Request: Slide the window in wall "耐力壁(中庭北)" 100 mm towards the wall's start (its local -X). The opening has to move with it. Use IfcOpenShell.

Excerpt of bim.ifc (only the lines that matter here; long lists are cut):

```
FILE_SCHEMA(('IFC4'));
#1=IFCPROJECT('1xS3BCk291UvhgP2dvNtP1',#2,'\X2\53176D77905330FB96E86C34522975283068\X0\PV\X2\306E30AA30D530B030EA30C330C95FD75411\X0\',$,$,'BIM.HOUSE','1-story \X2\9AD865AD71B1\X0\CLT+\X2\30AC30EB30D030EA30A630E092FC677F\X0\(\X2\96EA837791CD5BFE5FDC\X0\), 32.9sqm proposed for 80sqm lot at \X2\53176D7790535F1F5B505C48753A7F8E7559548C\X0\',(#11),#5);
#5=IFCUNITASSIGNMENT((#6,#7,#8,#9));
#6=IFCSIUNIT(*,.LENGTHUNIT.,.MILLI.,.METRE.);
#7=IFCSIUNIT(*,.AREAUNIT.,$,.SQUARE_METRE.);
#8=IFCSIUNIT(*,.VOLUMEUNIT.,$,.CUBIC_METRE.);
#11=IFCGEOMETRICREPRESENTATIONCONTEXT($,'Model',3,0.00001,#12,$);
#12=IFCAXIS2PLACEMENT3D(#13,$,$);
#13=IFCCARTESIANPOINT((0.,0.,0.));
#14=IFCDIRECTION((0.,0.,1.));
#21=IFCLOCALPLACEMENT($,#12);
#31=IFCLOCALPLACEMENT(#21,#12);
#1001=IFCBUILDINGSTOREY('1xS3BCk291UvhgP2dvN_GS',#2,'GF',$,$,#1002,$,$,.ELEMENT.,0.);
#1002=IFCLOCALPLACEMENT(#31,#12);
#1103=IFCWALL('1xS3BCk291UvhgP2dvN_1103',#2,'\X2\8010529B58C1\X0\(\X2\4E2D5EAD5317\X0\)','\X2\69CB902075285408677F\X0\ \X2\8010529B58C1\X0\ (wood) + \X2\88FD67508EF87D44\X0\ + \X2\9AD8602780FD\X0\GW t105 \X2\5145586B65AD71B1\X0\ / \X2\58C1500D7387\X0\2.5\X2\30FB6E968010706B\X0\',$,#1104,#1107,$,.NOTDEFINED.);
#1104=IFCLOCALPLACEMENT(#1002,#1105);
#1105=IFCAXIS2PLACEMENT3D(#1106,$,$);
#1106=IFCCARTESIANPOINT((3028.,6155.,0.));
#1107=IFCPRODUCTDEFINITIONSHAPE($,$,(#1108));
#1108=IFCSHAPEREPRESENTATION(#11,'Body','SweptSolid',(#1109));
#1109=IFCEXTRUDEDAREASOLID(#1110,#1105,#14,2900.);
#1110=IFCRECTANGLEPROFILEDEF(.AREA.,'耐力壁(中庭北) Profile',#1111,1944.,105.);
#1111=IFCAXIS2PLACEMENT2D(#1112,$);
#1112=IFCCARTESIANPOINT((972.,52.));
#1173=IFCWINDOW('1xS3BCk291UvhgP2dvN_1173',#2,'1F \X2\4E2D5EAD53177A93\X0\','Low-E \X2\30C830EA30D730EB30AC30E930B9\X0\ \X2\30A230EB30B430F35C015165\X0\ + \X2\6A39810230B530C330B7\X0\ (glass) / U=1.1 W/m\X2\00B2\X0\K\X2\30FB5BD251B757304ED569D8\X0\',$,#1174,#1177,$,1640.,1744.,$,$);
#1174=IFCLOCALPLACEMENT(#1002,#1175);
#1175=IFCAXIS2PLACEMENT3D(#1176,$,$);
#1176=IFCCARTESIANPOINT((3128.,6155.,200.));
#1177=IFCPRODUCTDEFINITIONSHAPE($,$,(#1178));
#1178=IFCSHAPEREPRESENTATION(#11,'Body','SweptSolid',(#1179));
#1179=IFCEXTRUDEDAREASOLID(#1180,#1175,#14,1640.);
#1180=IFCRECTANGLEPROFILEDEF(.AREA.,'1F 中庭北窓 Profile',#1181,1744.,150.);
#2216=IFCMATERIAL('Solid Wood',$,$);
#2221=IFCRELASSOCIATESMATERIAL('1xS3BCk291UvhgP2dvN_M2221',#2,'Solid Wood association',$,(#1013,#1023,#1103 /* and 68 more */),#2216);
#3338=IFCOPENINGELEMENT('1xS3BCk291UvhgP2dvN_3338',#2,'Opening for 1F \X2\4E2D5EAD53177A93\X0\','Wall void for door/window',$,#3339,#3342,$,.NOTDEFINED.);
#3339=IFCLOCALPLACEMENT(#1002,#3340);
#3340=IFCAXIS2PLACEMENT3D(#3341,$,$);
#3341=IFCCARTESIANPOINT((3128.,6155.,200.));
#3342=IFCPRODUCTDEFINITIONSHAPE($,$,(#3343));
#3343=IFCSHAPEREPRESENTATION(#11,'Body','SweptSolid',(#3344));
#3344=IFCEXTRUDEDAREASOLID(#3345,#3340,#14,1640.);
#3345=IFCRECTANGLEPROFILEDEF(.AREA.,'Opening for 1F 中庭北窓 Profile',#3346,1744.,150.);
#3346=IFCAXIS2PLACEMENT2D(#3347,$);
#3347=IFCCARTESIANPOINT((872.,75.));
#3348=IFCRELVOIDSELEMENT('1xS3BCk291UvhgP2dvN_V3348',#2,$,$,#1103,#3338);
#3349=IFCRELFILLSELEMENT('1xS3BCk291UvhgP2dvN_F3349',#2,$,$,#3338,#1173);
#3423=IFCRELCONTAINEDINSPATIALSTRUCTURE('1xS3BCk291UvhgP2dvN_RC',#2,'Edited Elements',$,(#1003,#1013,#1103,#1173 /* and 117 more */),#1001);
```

```python
import ifcopenshell
import ifcopenshell.api.geometry
import ifcopenshell.util.placement
import ifcopenshell.util.unit

model = ifcopenshell.open("bim.ifc")
unit_scale = ifcopenshell.util.unit.calculate_unit_scale(model)

window = model.by_guid("1xS3BCk291UvhgP2dvN_1173")
opening = window.FillsVoids[0].RelatingOpeningElement
wall = opening.VoidsElements[0].RelatingBuildingElement

wall_matrix = ifcopenshell.util.placement.get_local_placement(wall.ObjectPlacement)
shift = wall_matrix[:3, 0] * -0.1 / unit_scale
before = ifcopenshell.util.placement.get_local_placement(window.ObjectPlacement)[:3, 3].copy()

# The window is not placed relative to its opening, so move both.
for product in (opening, window):
    matrix = ifcopenshell.util.placement.get_local_placement(product.ObjectPlacement)
    matrix[:3, 3] += shift
    ifcopenshell.api.geometry.edit_object_placement(model, product=product, matrix=matrix, is_si=False)

after = ifcopenshell.util.placement.get_local_placement(window.ObjectPlacement)[:3, 3]
print("window moved by", (after - before).round(3) + 0.0)

model.write("bim_updated.ifc")
```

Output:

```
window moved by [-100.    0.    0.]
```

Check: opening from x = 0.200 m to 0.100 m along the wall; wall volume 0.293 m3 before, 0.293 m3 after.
